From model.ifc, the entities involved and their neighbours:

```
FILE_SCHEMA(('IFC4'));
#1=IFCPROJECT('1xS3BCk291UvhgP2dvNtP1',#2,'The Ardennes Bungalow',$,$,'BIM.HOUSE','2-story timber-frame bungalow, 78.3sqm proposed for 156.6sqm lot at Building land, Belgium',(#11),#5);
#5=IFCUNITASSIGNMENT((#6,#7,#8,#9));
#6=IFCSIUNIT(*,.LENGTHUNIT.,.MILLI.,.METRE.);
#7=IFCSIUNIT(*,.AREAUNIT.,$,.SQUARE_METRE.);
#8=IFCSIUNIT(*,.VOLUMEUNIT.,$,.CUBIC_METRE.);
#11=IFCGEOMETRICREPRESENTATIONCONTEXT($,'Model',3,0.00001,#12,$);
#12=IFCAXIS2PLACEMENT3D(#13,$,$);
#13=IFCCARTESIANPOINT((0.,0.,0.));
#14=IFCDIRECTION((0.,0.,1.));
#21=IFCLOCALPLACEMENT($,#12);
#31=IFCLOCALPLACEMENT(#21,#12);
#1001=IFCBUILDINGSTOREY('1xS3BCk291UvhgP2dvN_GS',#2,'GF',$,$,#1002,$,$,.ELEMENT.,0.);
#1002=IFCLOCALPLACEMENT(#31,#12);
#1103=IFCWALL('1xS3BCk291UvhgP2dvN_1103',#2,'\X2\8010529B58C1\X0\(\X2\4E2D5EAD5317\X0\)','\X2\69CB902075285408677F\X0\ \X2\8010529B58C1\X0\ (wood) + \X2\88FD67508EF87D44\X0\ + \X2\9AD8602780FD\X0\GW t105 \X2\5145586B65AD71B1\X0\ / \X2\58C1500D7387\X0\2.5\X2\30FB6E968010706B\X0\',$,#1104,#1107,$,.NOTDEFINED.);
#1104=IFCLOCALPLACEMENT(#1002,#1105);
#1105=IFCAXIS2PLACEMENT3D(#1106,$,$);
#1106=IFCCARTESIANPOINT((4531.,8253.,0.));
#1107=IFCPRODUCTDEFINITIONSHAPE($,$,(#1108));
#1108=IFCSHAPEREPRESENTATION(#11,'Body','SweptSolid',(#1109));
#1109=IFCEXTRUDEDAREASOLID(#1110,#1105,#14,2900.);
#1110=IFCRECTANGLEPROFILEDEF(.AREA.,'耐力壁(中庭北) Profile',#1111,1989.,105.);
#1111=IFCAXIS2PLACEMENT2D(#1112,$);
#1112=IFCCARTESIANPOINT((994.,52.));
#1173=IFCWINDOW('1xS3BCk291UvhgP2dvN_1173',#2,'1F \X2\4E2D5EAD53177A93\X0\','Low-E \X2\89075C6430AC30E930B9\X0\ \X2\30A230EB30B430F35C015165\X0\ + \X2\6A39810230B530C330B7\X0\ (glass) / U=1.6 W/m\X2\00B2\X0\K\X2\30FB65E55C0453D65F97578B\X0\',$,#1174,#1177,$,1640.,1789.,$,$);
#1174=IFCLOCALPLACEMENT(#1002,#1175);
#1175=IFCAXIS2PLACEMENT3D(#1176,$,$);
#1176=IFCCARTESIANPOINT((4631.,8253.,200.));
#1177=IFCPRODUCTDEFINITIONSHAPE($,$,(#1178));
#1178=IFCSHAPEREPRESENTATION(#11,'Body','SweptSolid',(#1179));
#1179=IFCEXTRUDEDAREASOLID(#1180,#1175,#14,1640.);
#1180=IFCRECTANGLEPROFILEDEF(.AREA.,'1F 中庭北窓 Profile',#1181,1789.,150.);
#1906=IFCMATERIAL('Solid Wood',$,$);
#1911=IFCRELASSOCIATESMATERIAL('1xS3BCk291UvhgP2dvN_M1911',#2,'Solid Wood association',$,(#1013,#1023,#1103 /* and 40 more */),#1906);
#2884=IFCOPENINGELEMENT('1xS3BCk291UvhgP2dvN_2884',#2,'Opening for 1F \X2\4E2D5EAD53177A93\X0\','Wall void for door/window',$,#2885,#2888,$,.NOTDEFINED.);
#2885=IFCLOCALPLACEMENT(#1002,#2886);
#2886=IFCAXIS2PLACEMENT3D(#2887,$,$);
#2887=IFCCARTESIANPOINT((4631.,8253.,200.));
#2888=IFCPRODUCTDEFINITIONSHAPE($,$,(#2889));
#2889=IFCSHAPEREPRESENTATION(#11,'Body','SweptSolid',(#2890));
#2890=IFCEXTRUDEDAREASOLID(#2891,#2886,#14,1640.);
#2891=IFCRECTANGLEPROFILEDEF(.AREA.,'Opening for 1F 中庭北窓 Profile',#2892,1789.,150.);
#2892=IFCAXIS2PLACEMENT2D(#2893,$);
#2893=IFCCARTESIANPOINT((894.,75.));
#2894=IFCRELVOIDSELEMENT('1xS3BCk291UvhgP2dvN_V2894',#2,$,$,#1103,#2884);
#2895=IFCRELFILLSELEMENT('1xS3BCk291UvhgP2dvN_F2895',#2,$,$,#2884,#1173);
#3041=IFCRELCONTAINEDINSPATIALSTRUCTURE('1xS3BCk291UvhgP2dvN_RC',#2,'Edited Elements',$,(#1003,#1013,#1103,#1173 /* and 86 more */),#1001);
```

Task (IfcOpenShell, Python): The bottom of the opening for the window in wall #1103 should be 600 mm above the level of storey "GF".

```python
import numpy as np
import ifcopenshell
import ifcopenshell.api.geometry
import ifcopenshell.geom
import ifcopenshell.util.element
import ifcopenshell.util.placement
import ifcopenshell.util.shape
import ifcopenshell.util.unit

model = ifcopenshell.open("model.ifc")
unit_scale = ifcopenshell.util.unit.calculate_unit_scale(model)

window = model.by_guid("1xS3BCk291UvhgP2dvN_1173")
opening = window.FillsVoids[0].RelatingOpeningElement
storey = ifcopenshell.util.element.get_container(window, ifc_class="IfcBuildingStorey")
level = ifcopenshell.util.placement.get_local_placement(storey.ObjectPlacement)[2, 3]

# The opening's origin need not be at the sill, so measure its lowest point.
shape = ifcopenshell.geom.create_shape(ifcopenshell.geom.settings(), opening)
bottom = ifcopenshell.util.shape.get_shape_bottom_elevation(shape, shape.geometry) / unit_scale
dz = level + 600.0 - bottom

shift = np.array([0.0, 0.0, dz])
# The window is not placed relative to its opening, so move both.
for product in (opening, window):
    matrix = ifcopenshell.util.placement.get_local_placement(product.ObjectPlacement)
    matrix[:3, 3] += shift
    ifcopenshell.api.geometry.edit_object_placement(model, product=product, matrix=matrix, is_si=False)

print(f"moved by {dz * unit_scale:+.3f} m")

model.write("model-out.ifc")
```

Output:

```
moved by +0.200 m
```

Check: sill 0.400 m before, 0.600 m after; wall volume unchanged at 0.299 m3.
